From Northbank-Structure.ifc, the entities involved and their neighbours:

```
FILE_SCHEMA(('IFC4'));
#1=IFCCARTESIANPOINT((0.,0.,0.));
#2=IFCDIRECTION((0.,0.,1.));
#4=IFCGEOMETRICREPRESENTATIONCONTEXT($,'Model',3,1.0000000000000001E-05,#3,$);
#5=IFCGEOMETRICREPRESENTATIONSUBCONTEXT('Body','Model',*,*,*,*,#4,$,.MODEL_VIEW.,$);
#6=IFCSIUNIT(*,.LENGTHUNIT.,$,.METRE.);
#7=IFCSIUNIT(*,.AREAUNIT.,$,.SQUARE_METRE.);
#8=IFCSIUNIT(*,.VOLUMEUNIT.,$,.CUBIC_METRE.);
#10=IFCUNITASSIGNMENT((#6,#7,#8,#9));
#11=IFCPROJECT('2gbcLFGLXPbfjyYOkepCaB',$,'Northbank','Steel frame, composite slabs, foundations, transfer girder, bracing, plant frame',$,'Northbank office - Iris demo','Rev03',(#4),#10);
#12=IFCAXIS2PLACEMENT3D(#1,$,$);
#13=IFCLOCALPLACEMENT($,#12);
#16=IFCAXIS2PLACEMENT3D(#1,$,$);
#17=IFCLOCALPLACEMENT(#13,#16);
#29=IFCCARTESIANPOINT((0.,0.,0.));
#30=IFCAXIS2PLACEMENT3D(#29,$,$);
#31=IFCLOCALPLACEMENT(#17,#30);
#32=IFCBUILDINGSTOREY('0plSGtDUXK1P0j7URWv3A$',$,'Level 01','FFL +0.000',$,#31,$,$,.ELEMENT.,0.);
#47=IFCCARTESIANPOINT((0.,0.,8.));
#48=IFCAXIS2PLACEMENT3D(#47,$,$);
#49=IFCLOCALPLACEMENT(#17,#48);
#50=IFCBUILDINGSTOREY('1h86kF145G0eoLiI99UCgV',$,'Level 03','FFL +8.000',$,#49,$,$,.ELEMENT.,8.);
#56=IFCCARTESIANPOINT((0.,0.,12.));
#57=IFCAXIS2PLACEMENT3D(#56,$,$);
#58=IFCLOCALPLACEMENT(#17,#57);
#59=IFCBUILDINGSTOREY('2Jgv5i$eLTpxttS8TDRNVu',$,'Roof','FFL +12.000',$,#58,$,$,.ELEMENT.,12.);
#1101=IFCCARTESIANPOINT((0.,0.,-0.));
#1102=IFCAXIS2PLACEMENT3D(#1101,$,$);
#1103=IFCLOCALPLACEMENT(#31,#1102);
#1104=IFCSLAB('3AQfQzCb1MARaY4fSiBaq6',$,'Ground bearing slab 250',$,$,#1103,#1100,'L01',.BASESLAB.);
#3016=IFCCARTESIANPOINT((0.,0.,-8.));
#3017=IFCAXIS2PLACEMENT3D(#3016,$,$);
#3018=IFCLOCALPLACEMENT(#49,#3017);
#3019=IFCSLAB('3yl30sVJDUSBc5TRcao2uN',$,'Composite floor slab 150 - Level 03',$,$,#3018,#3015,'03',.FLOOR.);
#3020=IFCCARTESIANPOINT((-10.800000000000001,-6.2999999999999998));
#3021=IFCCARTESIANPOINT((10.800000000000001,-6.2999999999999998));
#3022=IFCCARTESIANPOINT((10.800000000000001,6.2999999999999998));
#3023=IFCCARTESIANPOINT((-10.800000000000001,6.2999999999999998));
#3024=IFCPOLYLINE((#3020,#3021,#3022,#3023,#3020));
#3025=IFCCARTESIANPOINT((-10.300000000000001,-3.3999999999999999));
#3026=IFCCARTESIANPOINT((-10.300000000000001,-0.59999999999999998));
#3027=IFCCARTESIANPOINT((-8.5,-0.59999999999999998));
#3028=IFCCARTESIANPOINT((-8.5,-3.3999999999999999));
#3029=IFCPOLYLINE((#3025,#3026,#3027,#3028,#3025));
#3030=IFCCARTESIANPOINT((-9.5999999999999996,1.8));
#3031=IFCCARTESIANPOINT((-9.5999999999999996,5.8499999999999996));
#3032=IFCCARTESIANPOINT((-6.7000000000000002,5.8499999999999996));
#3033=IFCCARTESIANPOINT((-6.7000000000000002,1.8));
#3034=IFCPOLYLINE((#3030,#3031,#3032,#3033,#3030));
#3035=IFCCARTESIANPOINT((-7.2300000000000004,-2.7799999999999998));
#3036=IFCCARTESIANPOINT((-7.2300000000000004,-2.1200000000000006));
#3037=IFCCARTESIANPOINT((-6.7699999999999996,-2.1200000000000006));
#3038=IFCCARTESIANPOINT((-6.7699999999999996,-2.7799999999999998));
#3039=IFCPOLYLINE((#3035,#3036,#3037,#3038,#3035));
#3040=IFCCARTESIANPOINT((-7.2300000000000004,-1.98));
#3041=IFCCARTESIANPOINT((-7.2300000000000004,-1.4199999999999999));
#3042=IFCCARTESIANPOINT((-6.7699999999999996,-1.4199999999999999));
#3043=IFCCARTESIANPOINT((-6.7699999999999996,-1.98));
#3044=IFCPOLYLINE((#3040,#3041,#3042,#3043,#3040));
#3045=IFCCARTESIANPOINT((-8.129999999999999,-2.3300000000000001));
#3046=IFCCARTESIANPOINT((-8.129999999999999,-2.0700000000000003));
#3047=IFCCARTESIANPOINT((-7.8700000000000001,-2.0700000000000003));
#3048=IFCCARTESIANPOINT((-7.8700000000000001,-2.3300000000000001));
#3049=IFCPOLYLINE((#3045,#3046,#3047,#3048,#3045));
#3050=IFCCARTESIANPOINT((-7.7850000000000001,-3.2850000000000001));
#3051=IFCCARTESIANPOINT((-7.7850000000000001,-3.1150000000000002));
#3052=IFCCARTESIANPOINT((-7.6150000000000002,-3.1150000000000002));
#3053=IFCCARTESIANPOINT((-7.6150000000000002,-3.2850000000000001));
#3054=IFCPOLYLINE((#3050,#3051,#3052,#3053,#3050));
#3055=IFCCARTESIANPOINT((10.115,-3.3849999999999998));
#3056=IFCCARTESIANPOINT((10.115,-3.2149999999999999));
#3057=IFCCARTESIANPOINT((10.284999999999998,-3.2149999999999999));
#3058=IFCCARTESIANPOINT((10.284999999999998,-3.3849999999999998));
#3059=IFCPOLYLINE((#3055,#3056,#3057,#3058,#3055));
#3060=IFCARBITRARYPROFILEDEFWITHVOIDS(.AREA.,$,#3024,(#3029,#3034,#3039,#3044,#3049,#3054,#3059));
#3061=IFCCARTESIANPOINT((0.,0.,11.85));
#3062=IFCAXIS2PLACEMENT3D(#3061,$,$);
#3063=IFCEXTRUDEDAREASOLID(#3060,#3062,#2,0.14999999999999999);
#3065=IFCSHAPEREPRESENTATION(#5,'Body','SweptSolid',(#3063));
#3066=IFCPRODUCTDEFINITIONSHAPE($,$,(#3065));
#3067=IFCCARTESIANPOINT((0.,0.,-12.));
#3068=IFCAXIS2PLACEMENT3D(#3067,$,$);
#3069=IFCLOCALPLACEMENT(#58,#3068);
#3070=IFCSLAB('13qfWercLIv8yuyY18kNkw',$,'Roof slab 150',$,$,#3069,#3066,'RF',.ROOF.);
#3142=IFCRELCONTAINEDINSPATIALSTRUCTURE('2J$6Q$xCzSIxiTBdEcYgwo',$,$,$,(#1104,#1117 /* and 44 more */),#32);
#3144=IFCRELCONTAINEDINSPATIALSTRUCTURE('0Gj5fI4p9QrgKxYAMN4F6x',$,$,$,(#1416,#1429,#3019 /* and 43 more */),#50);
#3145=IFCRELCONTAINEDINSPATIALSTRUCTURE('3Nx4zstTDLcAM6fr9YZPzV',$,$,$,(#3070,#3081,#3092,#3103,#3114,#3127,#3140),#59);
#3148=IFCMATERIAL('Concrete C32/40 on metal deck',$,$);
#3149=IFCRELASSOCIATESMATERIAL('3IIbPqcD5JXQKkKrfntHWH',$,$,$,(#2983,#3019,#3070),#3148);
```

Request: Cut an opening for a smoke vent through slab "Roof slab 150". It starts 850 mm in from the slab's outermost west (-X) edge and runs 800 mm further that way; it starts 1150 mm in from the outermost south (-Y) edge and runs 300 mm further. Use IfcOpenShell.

```python
import numpy as np
import ifcopenshell
import ifcopenshell.api.feature
import ifcopenshell.api.geometry
import ifcopenshell.api.root
import ifcopenshell.geom
import ifcopenshell.util.placement
import ifcopenshell.util.representation
import ifcopenshell.util.shape
import ifcopenshell.util.unit

model = ifcopenshell.open("Northbank-Structure.ifc")
unit_scale = ifcopenshell.util.unit.calculate_unit_scale(model)
settings = ifcopenshell.geom.settings()


def volume(element):
    """Net volume in cubic metres, openings subtracted."""
    shape = ifcopenshell.geom.create_shape(settings, element)
    return ifcopenshell.util.shape.get_volume(shape.geometry)


slab = model.by_guid("13qfWercLIv8yuyY18kNkw")
before = volume(slab)

# Extent in the slab's own axes, in metres. The edges named are its -X and -Y sides.
slab_shape = ifcopenshell.geom.create_shape(settings, slab)
vertices = ifcopenshell.util.shape.get_vertices(slab_shape.geometry)
x_min, y_min, bottom = vertices.min(axis=0)
top = vertices[:, 2].max()

opening = ifcopenshell.api.root.create_entity(model, ifc_class="IfcOpeningElement", name="Smoke vent opening", predefined_type="OPENING")
context = ifcopenshell.util.representation.get_context(model, "Model", "Body", "MODEL_VIEW")
width, depth = 0.8, 0.3
outline = [(0.0, 0.0), (width, 0.0), (width, depth), (0.0, depth), (0.0, 0.0)]
# Overshoot both faces by 50 mm so the cut is clean.
shape = ifcopenshell.api.geometry.add_slab_representation(
    model, context=context, depth=top - bottom + 0.1, polyline=outline
)
ifcopenshell.api.geometry.assign_representation(model, product=opening, representation=shape)

matrix = ifcopenshell.util.placement.get_local_placement(slab.ObjectPlacement)
matrix[:, 3] = matrix @ np.append(np.array([x_min + 0.85, y_min + 1.15, bottom - 0.05]) / unit_scale, 1.0)
ifcopenshell.api.geometry.edit_object_placement(model, product=opening, matrix=matrix, is_si=False)
ifcopenshell.api.feature.add_feature(model, feature=opening, element=slab)

after = volume(slab)

print(f"slab volume {before:.3f} -> {after:.3f} m3")

model.write("Northbank-Structure-out.ifc")
```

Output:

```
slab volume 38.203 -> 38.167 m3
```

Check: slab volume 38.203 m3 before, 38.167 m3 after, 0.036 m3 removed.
